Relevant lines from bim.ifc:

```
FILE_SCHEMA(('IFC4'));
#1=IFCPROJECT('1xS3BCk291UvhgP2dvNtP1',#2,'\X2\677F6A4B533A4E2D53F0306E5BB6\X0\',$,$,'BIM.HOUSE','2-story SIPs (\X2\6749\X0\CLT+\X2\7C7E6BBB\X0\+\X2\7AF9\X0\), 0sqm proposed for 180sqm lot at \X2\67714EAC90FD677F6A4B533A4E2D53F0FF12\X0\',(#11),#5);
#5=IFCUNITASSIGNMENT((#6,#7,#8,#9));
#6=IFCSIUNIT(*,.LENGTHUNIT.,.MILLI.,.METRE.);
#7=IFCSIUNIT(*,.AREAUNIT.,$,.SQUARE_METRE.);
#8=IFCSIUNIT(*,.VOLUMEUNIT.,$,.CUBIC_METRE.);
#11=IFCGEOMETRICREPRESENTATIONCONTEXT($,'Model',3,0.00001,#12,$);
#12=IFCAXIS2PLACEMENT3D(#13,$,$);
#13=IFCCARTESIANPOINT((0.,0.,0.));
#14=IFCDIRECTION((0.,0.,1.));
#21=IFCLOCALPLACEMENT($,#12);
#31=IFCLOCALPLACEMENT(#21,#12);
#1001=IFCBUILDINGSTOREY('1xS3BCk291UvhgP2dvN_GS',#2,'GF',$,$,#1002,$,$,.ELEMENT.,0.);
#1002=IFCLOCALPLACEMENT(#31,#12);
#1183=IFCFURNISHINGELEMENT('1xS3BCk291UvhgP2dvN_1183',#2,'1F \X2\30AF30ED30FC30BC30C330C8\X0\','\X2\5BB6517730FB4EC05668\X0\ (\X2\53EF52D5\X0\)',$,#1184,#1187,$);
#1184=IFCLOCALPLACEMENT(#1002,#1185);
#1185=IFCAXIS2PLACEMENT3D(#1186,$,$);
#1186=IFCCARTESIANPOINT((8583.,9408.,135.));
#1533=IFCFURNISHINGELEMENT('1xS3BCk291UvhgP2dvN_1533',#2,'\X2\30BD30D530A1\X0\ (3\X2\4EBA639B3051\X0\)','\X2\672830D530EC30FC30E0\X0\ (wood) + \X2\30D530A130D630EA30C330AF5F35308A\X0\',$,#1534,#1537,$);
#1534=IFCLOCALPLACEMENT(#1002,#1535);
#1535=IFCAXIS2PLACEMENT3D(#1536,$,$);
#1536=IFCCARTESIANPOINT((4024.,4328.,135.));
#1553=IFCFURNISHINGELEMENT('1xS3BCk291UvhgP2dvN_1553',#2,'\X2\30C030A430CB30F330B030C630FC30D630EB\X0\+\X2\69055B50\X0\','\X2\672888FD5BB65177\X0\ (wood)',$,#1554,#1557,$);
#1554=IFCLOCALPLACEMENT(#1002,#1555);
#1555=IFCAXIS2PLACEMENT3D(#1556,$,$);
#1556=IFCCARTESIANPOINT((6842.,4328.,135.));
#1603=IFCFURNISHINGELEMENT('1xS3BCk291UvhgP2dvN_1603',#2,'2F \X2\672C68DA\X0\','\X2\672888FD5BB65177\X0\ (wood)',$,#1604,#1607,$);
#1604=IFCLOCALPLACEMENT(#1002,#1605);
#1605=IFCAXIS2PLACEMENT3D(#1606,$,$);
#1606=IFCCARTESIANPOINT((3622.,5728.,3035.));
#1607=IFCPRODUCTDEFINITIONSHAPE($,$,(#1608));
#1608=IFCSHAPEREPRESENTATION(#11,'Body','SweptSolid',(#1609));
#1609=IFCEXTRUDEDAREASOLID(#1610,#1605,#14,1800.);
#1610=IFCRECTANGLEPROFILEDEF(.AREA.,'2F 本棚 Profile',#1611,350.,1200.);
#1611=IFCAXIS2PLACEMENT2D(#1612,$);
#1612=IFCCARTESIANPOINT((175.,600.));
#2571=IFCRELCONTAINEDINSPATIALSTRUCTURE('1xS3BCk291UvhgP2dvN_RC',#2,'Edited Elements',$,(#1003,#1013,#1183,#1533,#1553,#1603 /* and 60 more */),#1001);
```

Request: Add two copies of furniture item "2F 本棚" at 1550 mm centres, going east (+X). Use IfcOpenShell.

```python
import numpy as np
import ifcopenshell
import ifcopenshell.api.geometry
import ifcopenshell.api.root
import ifcopenshell.util.element
import ifcopenshell.util.placement

model = ifcopenshell.open("bim.ifc")


def reuse_history(source, copy):
    """copy_class also copies each property set's owner history, people and application; keep the originals."""
    for rel in copy.IsDefinedBy:
        if rel.is_a("IfcRelDefinesByProperties") and (history := rel.RelatingPropertyDefinition.OwnerHistory):
            rel.RelatingPropertyDefinition.OwnerHistory = source.OwnerHistory
            ifcopenshell.util.element.remove_deep2(model, history)


source = model.by_id(1603)
base = ifcopenshell.util.placement.get_local_placement(source.ObjectPlacement)
step = np.array([1.0, 0.0, 0.0]) * 1550.0

for i in range(1, 3):
    copy = ifcopenshell.api.root.copy_class(model, product=source)
    copy.Representation = ifcopenshell.util.element.copy_deep(
        model, source.Representation, exclude=["IfcGeometricRepresentationContext", "IfcRepresentationMap"]
    )
    reuse_history(source, copy)
    matrix = base.copy()
    matrix[:3, 3] += i * step
    print("added at", matrix[:3, 3].round(3) + 0.0)
    ifcopenshell.api.geometry.edit_object_placement(model, product=copy, matrix=matrix, is_si=False)

model.write("bim_v2.ifc")
```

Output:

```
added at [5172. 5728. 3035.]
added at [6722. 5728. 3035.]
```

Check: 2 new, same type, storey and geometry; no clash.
